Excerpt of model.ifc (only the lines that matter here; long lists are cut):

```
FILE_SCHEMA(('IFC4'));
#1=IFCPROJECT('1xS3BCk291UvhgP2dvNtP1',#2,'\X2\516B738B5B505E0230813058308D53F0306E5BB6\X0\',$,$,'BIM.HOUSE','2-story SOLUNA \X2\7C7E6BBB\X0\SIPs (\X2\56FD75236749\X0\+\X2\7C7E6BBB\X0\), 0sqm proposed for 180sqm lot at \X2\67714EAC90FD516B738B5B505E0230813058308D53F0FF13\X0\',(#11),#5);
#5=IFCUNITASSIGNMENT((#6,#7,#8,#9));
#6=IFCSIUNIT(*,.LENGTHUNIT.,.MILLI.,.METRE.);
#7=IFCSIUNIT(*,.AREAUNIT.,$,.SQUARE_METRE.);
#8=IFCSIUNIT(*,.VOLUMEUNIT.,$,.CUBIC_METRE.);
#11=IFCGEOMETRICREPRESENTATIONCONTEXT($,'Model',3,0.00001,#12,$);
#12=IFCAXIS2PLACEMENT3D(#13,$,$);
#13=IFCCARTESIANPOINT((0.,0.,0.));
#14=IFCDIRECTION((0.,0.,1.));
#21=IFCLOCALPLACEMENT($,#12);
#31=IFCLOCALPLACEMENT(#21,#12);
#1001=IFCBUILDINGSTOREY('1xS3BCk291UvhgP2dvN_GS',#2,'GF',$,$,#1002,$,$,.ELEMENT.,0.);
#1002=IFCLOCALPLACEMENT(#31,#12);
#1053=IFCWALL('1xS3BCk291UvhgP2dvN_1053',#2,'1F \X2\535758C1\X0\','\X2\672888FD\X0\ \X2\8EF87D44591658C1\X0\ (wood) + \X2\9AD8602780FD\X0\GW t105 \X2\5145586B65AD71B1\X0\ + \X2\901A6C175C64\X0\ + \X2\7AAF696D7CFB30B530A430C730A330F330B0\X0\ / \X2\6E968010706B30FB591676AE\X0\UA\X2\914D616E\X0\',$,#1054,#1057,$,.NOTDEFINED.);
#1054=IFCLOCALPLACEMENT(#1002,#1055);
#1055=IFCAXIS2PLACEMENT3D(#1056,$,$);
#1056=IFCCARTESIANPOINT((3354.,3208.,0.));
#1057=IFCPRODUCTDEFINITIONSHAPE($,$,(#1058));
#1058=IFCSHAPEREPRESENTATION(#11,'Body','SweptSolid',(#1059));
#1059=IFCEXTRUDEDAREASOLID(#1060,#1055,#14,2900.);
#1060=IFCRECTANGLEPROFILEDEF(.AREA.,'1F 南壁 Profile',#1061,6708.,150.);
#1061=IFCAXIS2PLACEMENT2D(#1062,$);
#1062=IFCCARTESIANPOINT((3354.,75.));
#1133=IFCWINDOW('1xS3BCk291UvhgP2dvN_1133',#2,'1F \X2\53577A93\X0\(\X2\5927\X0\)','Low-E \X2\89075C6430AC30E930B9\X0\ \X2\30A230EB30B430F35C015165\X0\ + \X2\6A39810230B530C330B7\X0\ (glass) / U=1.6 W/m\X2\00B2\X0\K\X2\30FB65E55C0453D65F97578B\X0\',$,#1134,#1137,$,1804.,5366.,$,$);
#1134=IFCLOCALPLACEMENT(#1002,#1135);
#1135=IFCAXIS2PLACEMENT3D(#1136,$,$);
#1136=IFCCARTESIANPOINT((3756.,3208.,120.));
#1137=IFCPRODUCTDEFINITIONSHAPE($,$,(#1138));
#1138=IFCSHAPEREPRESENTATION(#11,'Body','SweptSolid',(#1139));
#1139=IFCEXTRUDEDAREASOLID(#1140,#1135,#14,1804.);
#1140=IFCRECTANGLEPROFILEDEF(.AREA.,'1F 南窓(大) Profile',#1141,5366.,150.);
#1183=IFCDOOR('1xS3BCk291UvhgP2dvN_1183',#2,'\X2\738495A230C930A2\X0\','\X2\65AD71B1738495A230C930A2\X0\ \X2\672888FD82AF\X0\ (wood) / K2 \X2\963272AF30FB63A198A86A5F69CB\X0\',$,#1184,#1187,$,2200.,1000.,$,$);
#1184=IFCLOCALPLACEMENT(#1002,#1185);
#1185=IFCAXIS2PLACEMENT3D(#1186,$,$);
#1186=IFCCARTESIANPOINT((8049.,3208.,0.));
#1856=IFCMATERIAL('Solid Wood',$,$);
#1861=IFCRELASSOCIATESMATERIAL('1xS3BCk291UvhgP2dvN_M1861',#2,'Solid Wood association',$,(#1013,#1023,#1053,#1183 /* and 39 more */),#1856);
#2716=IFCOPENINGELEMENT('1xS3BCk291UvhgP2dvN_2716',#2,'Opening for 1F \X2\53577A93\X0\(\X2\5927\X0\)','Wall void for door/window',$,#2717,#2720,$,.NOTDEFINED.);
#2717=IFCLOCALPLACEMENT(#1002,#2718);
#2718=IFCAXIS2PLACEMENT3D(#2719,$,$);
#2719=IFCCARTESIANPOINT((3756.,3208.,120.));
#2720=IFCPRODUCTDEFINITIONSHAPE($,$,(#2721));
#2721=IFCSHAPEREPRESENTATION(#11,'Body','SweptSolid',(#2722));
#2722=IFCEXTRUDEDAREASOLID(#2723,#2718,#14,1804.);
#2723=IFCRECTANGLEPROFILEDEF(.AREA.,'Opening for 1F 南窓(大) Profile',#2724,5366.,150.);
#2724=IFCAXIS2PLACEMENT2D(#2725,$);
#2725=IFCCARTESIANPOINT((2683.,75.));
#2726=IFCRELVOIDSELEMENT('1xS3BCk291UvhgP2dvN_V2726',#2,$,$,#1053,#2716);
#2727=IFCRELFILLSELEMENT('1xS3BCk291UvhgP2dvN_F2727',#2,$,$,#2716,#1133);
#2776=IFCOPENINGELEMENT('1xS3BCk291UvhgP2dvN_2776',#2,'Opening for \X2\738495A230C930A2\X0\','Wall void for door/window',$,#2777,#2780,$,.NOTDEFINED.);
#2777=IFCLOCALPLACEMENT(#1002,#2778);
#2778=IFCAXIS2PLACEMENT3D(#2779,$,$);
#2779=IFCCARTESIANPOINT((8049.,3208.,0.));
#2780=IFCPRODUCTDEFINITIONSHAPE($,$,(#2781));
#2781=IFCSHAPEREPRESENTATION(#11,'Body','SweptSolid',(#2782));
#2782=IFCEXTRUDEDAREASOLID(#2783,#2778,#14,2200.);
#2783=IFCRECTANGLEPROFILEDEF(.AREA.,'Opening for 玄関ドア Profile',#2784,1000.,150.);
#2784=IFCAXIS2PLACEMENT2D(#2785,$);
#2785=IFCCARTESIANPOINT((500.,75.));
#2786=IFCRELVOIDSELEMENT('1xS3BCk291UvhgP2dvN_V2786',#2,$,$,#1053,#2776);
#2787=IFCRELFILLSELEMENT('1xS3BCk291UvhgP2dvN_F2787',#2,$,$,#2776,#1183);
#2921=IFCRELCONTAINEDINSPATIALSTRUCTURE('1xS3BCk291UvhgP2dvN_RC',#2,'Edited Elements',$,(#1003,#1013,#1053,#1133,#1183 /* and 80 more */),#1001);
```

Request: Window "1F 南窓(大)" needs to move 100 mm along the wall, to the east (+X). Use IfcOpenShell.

```python
import ifcopenshell
import ifcopenshell.api.geometry
import ifcopenshell.util.placement

model = ifcopenshell.open("model.ifc")

window = model.by_id(1133)
opening = window.FillsVoids[0].RelatingOpeningElement
wall = opening.VoidsElements[0].RelatingBuildingElement

wall_matrix = ifcopenshell.util.placement.get_local_placement(wall.ObjectPlacement)
shift = wall_matrix[:3, 0] * 100.0
before = ifcopenshell.util.placement.get_local_placement(window.ObjectPlacement)[:3, 3].copy()

# The window is not placed relative to its opening, so move both.
for product in (opening, window):
    matrix = ifcopenshell.util.placement.get_local_placement(product.ObjectPlacement)
    matrix[:3, 3] += shift
    ifcopenshell.api.geometry.edit_object_placement(model, product=product, matrix=matrix, is_si=False)

after = ifcopenshell.util.placement.get_local_placement(window.ObjectPlacement)[:3, 3]
print("window moved by", (after - before).round(3) + 0.0)

model.write("model_rev.ifc")
```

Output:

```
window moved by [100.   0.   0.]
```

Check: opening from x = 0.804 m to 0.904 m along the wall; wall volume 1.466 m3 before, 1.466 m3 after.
